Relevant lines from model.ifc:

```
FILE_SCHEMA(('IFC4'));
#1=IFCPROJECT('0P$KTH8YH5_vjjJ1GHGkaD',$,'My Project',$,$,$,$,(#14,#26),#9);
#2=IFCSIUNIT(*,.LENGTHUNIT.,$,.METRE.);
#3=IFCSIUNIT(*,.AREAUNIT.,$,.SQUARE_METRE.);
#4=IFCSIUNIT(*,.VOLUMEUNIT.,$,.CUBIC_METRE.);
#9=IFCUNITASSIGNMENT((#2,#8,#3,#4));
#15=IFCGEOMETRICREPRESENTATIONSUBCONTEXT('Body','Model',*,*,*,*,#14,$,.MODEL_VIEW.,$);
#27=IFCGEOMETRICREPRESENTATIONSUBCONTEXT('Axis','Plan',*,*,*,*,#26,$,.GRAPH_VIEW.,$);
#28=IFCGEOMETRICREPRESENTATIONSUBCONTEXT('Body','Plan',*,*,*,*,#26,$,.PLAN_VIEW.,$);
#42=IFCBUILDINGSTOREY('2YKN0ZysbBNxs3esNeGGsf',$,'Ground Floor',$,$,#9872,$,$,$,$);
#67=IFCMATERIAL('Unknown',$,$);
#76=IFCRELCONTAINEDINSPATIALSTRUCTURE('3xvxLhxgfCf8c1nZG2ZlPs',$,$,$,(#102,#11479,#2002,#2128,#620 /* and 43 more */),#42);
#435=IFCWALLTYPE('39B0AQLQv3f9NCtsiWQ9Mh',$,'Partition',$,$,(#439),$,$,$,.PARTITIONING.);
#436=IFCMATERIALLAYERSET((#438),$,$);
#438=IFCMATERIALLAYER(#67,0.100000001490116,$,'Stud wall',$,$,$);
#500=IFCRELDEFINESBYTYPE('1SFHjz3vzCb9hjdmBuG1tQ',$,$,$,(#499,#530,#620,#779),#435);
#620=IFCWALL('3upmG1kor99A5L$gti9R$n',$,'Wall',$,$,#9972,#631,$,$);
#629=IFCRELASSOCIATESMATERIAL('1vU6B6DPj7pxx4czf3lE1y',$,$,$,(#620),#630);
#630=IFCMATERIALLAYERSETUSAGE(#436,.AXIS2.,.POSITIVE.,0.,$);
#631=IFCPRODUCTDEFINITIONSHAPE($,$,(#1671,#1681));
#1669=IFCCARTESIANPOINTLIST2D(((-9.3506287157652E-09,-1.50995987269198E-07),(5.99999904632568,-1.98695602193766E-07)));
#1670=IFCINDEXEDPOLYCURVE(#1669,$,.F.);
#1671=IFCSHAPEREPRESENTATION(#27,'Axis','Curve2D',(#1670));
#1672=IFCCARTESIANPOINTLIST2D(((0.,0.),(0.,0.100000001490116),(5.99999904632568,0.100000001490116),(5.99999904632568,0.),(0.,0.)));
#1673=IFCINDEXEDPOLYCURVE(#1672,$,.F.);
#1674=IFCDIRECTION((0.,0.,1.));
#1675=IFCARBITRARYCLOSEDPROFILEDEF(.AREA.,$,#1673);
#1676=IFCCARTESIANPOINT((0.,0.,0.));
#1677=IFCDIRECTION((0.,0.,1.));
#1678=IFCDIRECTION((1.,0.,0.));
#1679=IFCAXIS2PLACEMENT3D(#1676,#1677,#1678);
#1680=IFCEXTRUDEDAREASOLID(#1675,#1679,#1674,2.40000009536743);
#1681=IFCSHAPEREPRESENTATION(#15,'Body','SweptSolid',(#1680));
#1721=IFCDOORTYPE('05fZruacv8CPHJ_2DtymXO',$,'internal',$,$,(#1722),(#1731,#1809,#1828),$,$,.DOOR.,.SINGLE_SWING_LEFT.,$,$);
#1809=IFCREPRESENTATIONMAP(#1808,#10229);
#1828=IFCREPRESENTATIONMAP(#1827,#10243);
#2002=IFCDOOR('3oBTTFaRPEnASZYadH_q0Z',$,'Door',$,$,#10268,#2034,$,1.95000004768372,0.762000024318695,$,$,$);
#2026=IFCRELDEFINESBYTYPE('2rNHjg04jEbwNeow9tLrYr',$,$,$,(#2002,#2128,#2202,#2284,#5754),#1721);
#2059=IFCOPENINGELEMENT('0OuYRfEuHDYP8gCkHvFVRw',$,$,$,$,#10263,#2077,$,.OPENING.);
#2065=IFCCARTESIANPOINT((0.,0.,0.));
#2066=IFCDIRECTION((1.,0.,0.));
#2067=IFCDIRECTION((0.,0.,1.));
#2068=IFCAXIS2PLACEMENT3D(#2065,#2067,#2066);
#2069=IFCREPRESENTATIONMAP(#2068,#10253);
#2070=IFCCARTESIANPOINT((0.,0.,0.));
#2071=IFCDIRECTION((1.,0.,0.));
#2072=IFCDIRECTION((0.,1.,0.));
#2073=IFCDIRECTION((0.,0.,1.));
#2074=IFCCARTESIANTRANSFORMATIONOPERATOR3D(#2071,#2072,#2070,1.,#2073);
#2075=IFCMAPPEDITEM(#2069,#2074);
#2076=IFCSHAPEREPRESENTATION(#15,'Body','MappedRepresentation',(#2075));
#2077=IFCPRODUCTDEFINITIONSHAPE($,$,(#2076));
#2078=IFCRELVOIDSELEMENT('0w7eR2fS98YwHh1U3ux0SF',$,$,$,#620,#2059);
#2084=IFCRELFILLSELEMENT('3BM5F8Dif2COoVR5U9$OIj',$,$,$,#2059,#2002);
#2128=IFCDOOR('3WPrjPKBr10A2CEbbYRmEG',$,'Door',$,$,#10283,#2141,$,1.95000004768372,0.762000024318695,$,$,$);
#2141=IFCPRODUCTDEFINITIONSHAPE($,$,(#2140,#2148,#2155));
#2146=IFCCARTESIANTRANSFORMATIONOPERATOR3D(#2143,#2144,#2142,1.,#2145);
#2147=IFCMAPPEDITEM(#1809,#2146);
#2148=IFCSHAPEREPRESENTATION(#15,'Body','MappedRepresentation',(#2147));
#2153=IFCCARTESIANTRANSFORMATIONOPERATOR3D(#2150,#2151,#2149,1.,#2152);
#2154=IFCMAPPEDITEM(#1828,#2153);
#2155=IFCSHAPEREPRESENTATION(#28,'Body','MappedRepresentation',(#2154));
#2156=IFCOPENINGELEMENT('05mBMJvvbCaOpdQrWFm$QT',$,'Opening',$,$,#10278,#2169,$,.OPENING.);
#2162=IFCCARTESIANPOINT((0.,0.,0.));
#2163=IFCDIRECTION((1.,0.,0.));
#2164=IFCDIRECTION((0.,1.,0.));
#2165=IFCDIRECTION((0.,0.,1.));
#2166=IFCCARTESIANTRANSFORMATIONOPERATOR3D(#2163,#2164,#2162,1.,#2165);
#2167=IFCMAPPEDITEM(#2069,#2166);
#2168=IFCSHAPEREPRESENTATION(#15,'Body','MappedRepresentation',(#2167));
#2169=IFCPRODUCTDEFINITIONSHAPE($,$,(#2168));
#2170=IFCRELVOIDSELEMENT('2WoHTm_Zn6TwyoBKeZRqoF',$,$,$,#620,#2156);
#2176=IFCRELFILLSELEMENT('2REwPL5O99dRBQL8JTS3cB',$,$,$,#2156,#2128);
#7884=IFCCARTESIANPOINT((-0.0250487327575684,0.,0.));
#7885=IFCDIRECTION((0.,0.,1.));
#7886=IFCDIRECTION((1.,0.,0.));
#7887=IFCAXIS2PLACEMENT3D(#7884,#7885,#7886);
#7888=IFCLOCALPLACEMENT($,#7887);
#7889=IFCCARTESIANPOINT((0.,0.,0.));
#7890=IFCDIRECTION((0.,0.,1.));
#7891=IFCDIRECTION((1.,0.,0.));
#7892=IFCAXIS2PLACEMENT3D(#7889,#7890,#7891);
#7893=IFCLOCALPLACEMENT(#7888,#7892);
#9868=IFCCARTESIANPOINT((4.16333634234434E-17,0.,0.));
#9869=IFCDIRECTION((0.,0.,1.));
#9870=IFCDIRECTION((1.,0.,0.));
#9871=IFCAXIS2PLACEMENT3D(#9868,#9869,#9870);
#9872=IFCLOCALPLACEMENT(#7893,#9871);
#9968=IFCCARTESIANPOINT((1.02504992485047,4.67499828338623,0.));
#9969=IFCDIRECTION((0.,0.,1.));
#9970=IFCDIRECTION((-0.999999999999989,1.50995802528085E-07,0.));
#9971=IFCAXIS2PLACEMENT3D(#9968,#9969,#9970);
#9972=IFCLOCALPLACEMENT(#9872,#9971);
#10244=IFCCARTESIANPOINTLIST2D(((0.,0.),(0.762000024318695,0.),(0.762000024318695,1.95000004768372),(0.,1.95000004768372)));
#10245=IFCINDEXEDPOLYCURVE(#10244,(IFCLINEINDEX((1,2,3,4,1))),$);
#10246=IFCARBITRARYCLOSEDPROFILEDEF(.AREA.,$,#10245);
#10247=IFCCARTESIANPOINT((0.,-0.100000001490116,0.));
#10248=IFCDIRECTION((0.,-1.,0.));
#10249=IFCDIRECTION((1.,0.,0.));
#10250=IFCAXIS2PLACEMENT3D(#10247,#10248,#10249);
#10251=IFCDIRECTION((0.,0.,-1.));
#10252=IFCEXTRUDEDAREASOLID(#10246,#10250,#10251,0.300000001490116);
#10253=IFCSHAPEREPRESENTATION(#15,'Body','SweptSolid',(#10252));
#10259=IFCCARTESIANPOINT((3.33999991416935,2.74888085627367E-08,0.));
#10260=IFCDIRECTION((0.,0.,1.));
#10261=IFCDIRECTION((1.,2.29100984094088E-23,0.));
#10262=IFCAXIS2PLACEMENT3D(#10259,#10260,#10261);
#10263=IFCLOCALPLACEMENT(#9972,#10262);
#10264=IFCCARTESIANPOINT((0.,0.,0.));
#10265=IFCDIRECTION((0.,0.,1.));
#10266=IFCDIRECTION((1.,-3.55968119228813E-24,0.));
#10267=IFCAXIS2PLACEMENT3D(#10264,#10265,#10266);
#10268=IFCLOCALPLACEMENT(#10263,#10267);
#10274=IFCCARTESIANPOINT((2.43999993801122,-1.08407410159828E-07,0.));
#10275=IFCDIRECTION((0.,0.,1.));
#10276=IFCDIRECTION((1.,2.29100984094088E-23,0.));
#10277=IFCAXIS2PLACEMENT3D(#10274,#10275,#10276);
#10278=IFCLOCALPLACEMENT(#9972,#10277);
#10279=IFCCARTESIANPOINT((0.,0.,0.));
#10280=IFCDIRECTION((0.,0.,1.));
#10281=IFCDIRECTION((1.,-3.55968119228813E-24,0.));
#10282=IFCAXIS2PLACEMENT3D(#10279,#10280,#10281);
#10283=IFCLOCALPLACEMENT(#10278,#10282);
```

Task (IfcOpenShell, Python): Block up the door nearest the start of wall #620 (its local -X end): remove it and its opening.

```python
import ifcopenshell
import ifcopenshell.api.feature
import ifcopenshell.api.root
import ifcopenshell.geom
import ifcopenshell.util.shape

model = ifcopenshell.open("model.ifc")
settings = ifcopenshell.geom.settings()


def volume(element):
    """Net volume in cubic metres, openings subtracted."""
    shape = ifcopenshell.geom.create_shape(settings, element)
    return ifcopenshell.util.shape.get_volume(shape.geometry)


door = model.by_guid("3WPrjPKBr10A2CEbbYRmEG")
opening = door.FillsVoids[0].RelatingOpeningElement
wall = opening.VoidsElements[0].RelatingBuildingElement
before = volume(wall)

ifcopenshell.api.root.remove_product(model, product=door)
ifcopenshell.api.feature.remove_feature(model, feature=opening)

after = volume(wall)

print(f"wall volume {before:.3f} -> {after:.3f} m3")

model.write("model_rev.ifc")
```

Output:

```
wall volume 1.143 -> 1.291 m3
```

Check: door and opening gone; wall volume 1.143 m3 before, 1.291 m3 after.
